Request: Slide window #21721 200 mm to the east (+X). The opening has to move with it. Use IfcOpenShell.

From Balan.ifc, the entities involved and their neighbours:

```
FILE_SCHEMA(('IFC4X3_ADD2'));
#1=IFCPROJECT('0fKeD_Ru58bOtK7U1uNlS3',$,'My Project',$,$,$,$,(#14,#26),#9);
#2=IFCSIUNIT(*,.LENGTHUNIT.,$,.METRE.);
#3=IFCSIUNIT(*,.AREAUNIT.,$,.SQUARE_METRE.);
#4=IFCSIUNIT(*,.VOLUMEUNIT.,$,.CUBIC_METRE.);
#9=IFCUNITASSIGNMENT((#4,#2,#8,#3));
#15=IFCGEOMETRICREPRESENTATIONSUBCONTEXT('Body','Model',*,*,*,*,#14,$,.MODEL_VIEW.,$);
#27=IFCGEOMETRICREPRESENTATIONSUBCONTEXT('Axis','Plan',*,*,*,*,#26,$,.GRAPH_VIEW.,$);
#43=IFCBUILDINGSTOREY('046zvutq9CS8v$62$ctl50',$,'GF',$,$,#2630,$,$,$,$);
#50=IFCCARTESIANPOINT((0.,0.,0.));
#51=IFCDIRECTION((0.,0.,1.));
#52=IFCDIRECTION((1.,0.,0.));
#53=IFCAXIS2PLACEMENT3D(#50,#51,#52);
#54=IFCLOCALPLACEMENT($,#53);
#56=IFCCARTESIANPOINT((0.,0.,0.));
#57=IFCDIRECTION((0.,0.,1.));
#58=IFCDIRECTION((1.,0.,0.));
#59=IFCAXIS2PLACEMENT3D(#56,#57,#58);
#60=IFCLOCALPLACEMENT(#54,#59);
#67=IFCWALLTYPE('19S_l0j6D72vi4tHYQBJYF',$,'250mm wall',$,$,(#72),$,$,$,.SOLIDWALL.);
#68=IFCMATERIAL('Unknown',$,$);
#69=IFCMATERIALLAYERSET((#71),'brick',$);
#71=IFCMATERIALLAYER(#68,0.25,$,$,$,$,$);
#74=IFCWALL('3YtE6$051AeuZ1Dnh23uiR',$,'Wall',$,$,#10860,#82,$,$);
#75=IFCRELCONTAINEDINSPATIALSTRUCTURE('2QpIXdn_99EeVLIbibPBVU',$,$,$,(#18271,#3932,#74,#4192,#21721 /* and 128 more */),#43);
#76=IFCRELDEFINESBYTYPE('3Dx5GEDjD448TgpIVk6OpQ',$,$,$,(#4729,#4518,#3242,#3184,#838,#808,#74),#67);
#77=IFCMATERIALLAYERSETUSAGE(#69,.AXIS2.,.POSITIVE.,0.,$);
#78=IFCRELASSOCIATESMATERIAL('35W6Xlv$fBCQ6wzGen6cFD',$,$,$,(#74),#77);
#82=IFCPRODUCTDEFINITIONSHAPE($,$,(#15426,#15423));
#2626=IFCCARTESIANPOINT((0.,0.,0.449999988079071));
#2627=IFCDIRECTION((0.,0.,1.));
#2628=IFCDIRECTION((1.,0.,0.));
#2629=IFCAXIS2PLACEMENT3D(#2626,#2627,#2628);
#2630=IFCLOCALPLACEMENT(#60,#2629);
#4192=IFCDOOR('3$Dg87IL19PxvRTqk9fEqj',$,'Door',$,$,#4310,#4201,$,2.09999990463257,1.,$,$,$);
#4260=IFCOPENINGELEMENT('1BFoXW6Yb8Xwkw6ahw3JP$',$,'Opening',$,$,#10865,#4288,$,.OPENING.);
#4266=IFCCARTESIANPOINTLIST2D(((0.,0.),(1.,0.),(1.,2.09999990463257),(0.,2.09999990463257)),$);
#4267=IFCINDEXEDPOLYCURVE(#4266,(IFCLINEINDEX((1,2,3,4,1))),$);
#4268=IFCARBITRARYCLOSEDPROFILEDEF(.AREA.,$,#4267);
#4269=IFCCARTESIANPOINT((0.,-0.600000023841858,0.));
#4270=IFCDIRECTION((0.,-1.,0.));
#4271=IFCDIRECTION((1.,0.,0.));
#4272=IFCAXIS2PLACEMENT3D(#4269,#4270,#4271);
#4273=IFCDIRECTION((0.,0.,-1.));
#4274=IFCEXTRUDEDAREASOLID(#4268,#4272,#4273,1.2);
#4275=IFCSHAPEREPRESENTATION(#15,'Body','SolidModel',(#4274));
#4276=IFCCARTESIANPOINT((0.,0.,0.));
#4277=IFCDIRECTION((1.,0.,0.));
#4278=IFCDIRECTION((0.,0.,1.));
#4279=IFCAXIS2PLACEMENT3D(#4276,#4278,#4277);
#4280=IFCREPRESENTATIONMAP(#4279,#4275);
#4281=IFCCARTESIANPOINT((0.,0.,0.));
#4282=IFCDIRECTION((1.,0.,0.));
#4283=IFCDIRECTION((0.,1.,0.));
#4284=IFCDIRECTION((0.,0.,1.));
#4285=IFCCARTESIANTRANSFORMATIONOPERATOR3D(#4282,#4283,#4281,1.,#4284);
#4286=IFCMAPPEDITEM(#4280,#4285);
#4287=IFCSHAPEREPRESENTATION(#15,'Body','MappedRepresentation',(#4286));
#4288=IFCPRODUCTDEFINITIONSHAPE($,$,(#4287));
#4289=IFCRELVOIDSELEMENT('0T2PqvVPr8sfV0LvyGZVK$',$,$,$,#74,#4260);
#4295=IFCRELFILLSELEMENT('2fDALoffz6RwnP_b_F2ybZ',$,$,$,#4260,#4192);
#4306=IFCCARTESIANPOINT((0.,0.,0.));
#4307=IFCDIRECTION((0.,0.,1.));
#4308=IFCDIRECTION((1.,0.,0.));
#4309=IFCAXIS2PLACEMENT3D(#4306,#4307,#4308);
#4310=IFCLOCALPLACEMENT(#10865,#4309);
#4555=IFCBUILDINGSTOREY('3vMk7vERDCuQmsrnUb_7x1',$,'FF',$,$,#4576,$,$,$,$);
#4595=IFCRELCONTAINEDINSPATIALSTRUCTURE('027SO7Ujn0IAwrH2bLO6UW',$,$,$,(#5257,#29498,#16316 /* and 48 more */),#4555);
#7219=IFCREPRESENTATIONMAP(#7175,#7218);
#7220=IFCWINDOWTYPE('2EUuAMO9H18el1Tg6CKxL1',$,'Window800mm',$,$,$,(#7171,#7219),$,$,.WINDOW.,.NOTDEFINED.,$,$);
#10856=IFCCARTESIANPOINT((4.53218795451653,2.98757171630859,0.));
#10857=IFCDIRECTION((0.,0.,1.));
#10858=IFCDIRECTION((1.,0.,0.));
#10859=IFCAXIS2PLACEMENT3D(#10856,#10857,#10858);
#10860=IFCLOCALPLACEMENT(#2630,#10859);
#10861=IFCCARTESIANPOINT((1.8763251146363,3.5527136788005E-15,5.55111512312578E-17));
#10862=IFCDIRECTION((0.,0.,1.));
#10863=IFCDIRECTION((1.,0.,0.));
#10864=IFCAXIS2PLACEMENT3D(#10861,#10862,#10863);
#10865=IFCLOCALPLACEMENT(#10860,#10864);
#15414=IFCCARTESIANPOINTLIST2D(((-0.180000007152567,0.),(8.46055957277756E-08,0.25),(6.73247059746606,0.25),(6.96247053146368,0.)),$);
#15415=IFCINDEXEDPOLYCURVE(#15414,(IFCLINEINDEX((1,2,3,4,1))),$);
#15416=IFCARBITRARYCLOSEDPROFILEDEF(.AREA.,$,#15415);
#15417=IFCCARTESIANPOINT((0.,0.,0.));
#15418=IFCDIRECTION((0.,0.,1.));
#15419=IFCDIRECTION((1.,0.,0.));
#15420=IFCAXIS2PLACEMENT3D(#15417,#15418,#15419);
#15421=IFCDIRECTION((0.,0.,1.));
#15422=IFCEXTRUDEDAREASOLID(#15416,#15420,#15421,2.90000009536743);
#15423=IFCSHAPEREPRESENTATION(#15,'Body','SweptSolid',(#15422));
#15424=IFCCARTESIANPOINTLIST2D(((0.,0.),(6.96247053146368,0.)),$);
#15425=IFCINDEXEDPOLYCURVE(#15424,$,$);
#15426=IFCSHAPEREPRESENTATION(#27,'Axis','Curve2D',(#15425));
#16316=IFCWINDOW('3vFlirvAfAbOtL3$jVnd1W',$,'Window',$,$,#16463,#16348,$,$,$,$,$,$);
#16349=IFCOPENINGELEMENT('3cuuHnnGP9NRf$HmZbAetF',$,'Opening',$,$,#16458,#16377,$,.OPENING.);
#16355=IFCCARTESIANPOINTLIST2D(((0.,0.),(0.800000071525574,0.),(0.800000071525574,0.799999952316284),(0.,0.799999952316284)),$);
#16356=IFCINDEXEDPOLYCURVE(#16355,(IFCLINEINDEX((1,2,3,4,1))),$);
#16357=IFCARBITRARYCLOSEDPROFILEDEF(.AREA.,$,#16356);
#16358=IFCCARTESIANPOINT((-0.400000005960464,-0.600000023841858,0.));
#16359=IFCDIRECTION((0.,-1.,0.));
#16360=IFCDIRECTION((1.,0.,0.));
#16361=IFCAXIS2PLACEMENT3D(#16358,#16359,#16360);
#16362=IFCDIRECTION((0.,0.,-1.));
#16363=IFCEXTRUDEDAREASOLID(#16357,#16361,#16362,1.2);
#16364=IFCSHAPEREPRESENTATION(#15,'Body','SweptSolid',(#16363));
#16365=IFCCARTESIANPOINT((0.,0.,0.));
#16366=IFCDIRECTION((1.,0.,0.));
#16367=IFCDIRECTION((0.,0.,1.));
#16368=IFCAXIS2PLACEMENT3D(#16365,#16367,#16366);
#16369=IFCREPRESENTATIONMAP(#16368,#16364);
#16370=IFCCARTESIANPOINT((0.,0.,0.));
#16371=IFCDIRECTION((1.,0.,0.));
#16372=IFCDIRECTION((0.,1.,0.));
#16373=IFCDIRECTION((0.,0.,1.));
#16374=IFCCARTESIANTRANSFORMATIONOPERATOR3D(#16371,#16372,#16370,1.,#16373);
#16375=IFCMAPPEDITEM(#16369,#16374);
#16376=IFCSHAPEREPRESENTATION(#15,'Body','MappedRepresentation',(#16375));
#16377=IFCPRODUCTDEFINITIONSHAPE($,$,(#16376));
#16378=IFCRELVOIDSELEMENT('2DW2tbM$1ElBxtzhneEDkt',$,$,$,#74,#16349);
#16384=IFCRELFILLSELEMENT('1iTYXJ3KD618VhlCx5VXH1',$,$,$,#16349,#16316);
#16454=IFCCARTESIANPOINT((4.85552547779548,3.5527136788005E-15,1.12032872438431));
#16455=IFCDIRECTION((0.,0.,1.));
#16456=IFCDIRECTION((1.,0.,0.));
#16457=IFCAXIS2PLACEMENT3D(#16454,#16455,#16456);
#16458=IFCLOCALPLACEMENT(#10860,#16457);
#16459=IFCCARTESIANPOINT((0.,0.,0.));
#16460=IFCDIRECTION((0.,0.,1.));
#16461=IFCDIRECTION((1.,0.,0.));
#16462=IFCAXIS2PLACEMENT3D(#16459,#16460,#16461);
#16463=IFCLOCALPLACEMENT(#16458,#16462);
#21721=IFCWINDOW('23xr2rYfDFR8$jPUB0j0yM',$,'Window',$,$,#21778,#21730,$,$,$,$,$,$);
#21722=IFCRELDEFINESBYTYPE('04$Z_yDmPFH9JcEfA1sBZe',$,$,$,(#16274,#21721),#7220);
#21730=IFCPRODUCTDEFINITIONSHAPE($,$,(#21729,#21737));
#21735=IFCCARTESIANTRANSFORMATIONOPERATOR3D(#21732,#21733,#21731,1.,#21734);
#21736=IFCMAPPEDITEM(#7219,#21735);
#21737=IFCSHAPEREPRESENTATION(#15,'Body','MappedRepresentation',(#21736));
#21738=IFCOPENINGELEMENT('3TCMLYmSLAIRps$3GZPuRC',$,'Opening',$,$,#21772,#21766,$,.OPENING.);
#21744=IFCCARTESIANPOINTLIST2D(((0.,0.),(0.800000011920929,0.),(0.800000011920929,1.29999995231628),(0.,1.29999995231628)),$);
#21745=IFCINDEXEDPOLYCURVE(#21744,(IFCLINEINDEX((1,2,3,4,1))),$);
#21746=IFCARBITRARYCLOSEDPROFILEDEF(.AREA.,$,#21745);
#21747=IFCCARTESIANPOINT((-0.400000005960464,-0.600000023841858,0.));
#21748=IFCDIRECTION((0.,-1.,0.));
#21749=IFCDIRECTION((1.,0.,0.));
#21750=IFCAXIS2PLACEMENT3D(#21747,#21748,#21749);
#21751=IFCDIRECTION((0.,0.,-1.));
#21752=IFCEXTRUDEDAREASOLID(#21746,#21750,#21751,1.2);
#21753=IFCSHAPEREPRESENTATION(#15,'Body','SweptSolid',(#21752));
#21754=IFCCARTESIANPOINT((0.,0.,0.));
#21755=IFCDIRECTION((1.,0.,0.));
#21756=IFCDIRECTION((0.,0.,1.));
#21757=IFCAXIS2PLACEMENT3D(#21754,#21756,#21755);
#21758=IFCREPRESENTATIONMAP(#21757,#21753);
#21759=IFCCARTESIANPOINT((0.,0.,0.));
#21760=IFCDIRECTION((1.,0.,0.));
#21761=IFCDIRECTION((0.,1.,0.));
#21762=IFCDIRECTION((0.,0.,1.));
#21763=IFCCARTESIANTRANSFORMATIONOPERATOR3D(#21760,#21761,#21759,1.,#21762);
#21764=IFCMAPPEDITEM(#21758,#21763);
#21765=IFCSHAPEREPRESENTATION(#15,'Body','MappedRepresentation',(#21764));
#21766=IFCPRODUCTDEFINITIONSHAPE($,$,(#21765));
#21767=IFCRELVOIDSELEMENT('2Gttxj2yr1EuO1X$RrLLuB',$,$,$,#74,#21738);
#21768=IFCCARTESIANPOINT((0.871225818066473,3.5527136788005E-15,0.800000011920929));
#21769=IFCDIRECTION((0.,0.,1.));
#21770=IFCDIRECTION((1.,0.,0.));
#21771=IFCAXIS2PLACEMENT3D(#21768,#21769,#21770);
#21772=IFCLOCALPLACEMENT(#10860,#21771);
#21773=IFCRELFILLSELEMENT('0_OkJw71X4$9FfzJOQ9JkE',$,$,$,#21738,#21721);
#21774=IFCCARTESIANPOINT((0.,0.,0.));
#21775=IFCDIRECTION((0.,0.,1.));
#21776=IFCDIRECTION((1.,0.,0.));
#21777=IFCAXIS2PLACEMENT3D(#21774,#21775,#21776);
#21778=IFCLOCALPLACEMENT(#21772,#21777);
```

```python
import ifcopenshell
import ifcopenshell.api.geometry
import ifcopenshell.util.placement
import ifcopenshell.util.unit

model = ifcopenshell.open("Balan.ifc")
unit_scale = ifcopenshell.util.unit.calculate_unit_scale(model)

window = model.by_guid("23xr2rYfDFR8$jPUB0j0yM")
opening = window.FillsVoids[0].RelatingOpeningElement
wall = opening.VoidsElements[0].RelatingBuildingElement

wall_matrix = ifcopenshell.util.placement.get_local_placement(wall.ObjectPlacement)
shift = wall_matrix[:3, 0] * 0.2 / unit_scale
before = ifcopenshell.util.placement.get_local_placement(window.ObjectPlacement)[:3, 3].copy()

# The window is placed relative to its opening, so it follows when the opening moves.
matrix = ifcopenshell.util.placement.get_local_placement(opening.ObjectPlacement)
matrix[:3, 3] += shift
ifcopenshell.api.geometry.edit_object_placement(
    model, product=opening, matrix=matrix, is_si=False, should_transform_children=True
)

after = ifcopenshell.util.placement.get_local_placement(window.ObjectPlacement)[:3, 3]
print("window moved by", (after - before).round(3) + 0.0)

model.write("Balan_rev.ifc")
```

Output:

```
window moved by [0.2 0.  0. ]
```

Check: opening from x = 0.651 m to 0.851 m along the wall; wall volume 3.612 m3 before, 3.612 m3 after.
